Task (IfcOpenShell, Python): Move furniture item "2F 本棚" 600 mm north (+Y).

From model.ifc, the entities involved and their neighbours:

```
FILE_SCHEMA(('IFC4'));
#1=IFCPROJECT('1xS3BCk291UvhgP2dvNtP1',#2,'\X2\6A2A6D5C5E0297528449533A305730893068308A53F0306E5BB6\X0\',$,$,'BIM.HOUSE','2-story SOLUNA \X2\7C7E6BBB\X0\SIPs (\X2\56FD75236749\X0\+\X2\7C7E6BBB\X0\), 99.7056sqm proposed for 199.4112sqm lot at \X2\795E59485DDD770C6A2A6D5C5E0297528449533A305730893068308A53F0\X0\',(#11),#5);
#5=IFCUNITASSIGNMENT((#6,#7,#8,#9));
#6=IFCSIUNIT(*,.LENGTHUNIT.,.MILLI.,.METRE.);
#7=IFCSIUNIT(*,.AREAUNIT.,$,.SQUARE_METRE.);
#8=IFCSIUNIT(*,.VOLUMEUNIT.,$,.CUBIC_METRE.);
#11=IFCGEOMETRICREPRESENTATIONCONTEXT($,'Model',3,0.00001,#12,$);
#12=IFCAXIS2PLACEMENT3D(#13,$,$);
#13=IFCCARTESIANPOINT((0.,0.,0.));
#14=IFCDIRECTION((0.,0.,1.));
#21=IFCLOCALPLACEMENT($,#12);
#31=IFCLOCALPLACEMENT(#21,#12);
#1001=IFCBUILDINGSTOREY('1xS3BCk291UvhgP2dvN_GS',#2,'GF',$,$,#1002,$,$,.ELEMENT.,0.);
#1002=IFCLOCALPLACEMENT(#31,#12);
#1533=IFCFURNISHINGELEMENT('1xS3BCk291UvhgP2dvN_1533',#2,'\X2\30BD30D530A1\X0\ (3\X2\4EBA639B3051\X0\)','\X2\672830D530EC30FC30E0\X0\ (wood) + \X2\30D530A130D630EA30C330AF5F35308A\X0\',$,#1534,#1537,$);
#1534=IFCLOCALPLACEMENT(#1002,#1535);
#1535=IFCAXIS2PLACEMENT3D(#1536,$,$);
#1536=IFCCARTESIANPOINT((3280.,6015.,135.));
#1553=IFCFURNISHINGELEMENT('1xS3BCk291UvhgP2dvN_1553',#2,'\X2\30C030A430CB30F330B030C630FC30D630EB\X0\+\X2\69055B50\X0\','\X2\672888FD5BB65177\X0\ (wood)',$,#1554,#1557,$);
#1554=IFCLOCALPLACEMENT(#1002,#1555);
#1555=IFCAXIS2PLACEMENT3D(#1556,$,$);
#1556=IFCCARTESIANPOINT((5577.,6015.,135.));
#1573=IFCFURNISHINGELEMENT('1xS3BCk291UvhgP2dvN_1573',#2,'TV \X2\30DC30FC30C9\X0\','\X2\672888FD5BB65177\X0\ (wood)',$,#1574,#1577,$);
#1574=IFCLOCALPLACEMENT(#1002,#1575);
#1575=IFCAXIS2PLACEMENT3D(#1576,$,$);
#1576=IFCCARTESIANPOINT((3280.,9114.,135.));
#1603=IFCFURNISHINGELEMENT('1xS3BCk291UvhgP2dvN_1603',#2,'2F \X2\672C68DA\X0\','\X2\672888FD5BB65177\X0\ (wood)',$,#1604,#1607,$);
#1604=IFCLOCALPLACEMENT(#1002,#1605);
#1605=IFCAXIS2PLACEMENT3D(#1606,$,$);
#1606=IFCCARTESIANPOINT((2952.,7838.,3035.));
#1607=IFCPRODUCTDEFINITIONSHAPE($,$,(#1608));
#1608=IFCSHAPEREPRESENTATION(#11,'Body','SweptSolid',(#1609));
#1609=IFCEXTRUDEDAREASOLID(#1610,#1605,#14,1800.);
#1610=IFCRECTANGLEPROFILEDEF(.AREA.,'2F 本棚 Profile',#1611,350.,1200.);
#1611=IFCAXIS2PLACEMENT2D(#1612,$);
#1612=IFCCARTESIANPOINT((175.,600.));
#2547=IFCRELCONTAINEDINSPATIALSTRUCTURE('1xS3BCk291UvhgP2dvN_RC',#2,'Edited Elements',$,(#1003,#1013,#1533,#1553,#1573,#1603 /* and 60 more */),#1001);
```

```python
import ifcopenshell
import ifcopenshell.api.geometry
import ifcopenshell.util.placement
import ifcopenshell.util.unit

model = ifcopenshell.open("model.ifc")
unit_scale = ifcopenshell.util.unit.calculate_unit_scale(model)

item = model.by_id(1603)
matrix = ifcopenshell.util.placement.get_local_placement(item.ObjectPlacement)
matrix[1, 3] += 0.6 / unit_scale
ifcopenshell.api.geometry.edit_object_placement(model, product=item, matrix=matrix, is_si=False)

print(ifcopenshell.util.placement.get_local_placement(item.ObjectPlacement).round(3) + 0.0)

model.write("model_rev.ifc")
```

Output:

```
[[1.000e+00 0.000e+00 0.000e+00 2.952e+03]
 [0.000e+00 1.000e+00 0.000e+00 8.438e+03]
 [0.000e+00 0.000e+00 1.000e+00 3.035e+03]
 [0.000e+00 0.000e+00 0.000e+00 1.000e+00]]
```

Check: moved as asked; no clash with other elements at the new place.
